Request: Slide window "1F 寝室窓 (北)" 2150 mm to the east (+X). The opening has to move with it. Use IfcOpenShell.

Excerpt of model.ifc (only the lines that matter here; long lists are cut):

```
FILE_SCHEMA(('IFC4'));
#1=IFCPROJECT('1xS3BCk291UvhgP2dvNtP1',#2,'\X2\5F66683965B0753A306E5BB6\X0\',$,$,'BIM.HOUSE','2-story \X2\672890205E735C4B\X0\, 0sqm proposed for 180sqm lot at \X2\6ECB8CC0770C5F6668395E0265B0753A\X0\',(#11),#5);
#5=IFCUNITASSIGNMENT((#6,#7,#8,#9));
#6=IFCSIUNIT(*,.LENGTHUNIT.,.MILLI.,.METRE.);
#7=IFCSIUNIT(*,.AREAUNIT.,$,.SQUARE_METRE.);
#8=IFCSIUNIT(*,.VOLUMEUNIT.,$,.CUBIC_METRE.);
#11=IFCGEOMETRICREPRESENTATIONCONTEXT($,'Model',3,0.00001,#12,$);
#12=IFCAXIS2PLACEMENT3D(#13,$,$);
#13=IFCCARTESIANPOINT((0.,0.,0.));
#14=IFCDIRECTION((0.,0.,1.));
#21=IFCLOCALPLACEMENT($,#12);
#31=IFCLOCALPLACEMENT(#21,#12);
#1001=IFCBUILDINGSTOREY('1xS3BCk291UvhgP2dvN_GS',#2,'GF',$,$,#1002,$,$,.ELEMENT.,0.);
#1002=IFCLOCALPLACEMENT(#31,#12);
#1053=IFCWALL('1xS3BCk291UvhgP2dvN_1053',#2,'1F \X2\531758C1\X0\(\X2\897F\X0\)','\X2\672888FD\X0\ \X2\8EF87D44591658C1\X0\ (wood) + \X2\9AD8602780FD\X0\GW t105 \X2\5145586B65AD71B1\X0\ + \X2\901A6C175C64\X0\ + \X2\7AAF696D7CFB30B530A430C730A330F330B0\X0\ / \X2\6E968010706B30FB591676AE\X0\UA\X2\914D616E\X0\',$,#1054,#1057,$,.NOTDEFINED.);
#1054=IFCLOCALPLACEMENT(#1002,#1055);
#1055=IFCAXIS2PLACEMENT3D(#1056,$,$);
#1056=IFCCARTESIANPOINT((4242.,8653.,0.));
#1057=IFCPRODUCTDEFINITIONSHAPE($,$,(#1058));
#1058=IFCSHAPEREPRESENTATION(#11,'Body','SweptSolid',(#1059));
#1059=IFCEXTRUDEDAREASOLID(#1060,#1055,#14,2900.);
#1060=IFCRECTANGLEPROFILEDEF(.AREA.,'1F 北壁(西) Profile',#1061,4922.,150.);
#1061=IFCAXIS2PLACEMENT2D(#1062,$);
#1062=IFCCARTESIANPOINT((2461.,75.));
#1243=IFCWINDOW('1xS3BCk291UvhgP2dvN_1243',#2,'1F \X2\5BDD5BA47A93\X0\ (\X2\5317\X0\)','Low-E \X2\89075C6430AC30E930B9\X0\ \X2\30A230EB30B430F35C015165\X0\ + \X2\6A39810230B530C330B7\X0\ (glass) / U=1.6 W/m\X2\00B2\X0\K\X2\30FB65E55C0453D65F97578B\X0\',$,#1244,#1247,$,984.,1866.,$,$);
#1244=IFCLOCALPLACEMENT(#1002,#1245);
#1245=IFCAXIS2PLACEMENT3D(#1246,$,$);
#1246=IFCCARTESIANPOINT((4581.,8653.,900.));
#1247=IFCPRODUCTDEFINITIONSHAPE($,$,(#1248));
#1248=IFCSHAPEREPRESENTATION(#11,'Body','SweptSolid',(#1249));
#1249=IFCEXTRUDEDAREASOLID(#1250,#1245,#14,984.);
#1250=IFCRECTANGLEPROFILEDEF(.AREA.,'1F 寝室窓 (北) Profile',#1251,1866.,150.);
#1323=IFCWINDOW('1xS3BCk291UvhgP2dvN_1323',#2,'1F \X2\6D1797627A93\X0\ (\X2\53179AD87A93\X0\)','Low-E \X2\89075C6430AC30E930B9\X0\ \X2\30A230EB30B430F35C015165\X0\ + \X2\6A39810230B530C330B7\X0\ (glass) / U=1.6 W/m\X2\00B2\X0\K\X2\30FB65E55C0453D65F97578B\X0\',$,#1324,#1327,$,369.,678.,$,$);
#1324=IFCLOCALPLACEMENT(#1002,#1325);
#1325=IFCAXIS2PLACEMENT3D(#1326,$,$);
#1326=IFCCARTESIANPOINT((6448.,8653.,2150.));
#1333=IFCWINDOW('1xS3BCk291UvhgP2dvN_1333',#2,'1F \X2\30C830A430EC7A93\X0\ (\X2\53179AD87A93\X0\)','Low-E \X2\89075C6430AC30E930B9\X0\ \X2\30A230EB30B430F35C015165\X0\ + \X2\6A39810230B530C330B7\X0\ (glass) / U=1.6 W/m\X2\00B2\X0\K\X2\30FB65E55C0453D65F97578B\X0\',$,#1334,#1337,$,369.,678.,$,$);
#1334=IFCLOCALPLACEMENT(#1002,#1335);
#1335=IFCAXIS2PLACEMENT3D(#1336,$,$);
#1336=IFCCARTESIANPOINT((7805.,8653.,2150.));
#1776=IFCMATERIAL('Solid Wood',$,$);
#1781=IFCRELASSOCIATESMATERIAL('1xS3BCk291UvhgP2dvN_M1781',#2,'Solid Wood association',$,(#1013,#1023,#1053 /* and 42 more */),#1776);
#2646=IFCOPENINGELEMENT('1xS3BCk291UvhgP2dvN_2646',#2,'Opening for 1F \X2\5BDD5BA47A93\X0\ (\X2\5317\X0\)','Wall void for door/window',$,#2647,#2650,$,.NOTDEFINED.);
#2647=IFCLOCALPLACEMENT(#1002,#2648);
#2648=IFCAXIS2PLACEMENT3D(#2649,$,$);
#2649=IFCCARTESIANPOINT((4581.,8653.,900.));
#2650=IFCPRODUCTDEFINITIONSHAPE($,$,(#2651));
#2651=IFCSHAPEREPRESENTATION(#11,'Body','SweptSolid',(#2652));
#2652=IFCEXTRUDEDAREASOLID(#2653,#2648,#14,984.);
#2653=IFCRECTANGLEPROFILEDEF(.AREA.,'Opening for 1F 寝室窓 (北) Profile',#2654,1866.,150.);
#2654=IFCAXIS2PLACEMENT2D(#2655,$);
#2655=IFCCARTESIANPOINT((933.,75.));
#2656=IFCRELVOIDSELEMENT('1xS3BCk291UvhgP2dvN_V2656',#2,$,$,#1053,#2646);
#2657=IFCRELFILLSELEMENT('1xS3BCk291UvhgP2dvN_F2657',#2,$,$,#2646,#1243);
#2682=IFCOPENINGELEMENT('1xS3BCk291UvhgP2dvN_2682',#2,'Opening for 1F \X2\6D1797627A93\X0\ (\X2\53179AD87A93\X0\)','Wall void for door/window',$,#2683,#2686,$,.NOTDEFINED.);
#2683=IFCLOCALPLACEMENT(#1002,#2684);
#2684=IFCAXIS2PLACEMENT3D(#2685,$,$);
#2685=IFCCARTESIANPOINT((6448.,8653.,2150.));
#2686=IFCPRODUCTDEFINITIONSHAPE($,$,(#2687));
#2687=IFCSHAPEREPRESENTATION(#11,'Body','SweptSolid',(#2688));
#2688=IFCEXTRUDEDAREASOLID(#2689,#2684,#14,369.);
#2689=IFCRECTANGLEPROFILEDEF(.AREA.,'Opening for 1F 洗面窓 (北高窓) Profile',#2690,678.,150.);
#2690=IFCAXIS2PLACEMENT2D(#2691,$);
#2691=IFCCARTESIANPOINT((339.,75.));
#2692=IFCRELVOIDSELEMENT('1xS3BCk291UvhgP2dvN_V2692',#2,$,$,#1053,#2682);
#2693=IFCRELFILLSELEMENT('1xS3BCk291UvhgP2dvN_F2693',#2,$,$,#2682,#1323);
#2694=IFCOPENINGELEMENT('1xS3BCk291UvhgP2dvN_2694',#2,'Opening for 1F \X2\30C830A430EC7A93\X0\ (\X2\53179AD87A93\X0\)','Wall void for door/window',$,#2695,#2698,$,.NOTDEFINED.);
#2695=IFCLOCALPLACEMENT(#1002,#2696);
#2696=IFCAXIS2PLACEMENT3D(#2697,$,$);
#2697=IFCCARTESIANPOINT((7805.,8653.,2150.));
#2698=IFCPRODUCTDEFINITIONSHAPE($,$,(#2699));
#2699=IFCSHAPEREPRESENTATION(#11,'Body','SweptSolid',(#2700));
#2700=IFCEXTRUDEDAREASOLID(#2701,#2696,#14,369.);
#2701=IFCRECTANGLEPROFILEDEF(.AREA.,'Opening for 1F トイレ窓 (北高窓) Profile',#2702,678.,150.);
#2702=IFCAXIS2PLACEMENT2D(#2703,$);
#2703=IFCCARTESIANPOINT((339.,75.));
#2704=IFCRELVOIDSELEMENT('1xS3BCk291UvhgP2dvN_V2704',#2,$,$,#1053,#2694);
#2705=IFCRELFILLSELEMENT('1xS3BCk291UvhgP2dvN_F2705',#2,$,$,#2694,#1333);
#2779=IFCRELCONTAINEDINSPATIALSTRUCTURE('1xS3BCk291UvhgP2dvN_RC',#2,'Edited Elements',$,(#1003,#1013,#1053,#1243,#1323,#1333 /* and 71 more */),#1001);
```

```python
import ifcopenshell
import ifcopenshell.api.geometry
import ifcopenshell.util.placement
import ifcopenshell.util.unit

model = ifcopenshell.open("model.ifc")
unit_scale = ifcopenshell.util.unit.calculate_unit_scale(model)

window = model.by_guid("1xS3BCk291UvhgP2dvN_1243")
opening = window.FillsVoids[0].RelatingOpeningElement
wall = opening.VoidsElements[0].RelatingBuildingElement

wall_matrix = ifcopenshell.util.placement.get_local_placement(wall.ObjectPlacement)
shift = wall_matrix[:3, 0] * 2.15 / unit_scale
before = ifcopenshell.util.placement.get_local_placement(window.ObjectPlacement)[:3, 3].copy()

# The window is not placed relative to its opening, so move both.
for product in (opening, window):
    matrix = ifcopenshell.util.placement.get_local_placement(product.ObjectPlacement)
    matrix[:3, 3] += shift
    ifcopenshell.api.geometry.edit_object_placement(model, product=product, matrix=matrix, is_si=False)

after = ifcopenshell.util.placement.get_local_placement(window.ObjectPlacement)[:3, 3]
print("window moved by", (after - before).round(3) + 0.0)

model.write("model_v2.ifc")
```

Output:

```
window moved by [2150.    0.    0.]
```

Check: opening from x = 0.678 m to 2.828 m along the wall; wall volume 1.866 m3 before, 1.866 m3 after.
